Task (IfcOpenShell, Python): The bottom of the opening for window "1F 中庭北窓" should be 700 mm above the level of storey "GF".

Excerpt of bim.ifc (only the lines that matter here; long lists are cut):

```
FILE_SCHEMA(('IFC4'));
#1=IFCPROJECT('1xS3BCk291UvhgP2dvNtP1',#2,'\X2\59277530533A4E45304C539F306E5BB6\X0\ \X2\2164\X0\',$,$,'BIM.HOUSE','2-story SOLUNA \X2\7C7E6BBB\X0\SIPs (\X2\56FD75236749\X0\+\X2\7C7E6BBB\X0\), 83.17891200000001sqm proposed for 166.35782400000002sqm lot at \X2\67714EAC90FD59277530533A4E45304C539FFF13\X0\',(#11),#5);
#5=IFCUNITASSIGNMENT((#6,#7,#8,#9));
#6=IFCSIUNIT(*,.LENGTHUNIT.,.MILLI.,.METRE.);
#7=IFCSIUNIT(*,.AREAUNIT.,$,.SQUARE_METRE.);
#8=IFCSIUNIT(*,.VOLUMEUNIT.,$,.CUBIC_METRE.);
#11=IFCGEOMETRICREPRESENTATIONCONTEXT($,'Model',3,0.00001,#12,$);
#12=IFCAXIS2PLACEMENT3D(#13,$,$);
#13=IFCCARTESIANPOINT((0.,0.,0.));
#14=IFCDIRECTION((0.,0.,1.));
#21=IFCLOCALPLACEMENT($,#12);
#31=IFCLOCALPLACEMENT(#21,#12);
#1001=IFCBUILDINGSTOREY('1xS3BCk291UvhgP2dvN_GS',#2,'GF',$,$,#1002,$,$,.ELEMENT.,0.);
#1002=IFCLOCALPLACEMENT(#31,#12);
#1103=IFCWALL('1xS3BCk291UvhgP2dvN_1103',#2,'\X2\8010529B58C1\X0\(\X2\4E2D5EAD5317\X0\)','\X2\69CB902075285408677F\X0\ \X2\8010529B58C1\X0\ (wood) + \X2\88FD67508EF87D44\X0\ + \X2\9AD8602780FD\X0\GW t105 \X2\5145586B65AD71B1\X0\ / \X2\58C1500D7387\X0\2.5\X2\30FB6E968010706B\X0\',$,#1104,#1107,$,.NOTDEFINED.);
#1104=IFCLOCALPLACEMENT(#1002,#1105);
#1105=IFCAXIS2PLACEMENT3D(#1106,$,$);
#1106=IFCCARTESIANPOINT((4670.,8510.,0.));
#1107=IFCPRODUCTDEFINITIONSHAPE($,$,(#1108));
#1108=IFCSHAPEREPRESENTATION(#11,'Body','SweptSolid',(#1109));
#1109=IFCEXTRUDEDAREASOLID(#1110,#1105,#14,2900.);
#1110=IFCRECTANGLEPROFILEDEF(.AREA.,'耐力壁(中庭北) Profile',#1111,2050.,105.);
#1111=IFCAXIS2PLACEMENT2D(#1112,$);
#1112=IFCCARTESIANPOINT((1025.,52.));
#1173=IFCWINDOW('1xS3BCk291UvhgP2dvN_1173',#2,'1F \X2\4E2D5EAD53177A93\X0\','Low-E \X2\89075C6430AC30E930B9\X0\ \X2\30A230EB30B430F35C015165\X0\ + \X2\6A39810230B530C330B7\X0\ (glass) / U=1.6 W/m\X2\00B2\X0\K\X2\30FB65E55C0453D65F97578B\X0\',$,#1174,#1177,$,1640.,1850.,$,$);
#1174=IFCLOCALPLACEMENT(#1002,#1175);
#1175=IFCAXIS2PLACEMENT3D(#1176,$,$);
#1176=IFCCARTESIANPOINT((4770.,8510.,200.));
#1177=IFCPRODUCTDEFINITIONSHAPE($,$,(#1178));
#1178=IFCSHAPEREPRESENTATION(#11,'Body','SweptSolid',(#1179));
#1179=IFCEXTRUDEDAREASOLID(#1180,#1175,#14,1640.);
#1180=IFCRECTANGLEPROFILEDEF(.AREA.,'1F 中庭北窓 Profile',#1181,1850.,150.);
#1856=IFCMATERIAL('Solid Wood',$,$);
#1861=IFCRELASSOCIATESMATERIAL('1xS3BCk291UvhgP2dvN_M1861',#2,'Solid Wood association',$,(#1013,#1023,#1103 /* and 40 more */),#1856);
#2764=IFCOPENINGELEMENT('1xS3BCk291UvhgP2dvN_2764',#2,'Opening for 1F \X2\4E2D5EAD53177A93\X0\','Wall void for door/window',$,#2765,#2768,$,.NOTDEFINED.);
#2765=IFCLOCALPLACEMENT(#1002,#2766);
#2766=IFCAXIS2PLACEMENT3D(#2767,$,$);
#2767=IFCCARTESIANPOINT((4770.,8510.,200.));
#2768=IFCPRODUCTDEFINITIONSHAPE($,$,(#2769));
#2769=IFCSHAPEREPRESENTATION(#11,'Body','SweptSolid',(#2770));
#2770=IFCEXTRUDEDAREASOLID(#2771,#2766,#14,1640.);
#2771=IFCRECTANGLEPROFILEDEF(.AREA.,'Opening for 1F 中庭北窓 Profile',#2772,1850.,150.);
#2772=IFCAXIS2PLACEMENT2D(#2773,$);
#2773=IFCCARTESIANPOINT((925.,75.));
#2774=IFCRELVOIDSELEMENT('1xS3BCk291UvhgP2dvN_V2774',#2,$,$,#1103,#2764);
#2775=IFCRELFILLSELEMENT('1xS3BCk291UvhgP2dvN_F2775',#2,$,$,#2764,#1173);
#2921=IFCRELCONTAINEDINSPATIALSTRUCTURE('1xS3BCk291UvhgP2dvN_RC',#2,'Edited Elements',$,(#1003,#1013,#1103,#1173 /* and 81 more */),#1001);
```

```python
import numpy as np
import ifcopenshell
import ifcopenshell.api.geometry
import ifcopenshell.geom
import ifcopenshell.util.element
import ifcopenshell.util.placement
import ifcopenshell.util.shape
import ifcopenshell.util.unit

model = ifcopenshell.open("bim.ifc")
unit_scale = ifcopenshell.util.unit.calculate_unit_scale(model)

window = model.by_guid("1xS3BCk291UvhgP2dvN_1173")
opening = window.FillsVoids[0].RelatingOpeningElement
storey = ifcopenshell.util.element.get_container(window, ifc_class="IfcBuildingStorey")
level = ifcopenshell.util.placement.get_local_placement(storey.ObjectPlacement)[2, 3]

# The opening's origin need not be at the sill, so measure its lowest point.
shape = ifcopenshell.geom.create_shape(ifcopenshell.geom.settings(), opening)
bottom = ifcopenshell.util.shape.get_shape_bottom_elevation(shape, shape.geometry) / unit_scale
dz = level + 0.7 / unit_scale - bottom

shift = np.array([0.0, 0.0, dz])
# The window is not placed relative to its opening, so move both.
for product in (opening, window):
    matrix = ifcopenshell.util.placement.get_local_placement(product.ObjectPlacement)
    matrix[:3, 3] += shift
    ifcopenshell.api.geometry.edit_object_placement(model, product=product, matrix=matrix, is_si=False)

print(f"moved by {dz * unit_scale:+.3f} m")

model.write("bim_edited.ifc")
```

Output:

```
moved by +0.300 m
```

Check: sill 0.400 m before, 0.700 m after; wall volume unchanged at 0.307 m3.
